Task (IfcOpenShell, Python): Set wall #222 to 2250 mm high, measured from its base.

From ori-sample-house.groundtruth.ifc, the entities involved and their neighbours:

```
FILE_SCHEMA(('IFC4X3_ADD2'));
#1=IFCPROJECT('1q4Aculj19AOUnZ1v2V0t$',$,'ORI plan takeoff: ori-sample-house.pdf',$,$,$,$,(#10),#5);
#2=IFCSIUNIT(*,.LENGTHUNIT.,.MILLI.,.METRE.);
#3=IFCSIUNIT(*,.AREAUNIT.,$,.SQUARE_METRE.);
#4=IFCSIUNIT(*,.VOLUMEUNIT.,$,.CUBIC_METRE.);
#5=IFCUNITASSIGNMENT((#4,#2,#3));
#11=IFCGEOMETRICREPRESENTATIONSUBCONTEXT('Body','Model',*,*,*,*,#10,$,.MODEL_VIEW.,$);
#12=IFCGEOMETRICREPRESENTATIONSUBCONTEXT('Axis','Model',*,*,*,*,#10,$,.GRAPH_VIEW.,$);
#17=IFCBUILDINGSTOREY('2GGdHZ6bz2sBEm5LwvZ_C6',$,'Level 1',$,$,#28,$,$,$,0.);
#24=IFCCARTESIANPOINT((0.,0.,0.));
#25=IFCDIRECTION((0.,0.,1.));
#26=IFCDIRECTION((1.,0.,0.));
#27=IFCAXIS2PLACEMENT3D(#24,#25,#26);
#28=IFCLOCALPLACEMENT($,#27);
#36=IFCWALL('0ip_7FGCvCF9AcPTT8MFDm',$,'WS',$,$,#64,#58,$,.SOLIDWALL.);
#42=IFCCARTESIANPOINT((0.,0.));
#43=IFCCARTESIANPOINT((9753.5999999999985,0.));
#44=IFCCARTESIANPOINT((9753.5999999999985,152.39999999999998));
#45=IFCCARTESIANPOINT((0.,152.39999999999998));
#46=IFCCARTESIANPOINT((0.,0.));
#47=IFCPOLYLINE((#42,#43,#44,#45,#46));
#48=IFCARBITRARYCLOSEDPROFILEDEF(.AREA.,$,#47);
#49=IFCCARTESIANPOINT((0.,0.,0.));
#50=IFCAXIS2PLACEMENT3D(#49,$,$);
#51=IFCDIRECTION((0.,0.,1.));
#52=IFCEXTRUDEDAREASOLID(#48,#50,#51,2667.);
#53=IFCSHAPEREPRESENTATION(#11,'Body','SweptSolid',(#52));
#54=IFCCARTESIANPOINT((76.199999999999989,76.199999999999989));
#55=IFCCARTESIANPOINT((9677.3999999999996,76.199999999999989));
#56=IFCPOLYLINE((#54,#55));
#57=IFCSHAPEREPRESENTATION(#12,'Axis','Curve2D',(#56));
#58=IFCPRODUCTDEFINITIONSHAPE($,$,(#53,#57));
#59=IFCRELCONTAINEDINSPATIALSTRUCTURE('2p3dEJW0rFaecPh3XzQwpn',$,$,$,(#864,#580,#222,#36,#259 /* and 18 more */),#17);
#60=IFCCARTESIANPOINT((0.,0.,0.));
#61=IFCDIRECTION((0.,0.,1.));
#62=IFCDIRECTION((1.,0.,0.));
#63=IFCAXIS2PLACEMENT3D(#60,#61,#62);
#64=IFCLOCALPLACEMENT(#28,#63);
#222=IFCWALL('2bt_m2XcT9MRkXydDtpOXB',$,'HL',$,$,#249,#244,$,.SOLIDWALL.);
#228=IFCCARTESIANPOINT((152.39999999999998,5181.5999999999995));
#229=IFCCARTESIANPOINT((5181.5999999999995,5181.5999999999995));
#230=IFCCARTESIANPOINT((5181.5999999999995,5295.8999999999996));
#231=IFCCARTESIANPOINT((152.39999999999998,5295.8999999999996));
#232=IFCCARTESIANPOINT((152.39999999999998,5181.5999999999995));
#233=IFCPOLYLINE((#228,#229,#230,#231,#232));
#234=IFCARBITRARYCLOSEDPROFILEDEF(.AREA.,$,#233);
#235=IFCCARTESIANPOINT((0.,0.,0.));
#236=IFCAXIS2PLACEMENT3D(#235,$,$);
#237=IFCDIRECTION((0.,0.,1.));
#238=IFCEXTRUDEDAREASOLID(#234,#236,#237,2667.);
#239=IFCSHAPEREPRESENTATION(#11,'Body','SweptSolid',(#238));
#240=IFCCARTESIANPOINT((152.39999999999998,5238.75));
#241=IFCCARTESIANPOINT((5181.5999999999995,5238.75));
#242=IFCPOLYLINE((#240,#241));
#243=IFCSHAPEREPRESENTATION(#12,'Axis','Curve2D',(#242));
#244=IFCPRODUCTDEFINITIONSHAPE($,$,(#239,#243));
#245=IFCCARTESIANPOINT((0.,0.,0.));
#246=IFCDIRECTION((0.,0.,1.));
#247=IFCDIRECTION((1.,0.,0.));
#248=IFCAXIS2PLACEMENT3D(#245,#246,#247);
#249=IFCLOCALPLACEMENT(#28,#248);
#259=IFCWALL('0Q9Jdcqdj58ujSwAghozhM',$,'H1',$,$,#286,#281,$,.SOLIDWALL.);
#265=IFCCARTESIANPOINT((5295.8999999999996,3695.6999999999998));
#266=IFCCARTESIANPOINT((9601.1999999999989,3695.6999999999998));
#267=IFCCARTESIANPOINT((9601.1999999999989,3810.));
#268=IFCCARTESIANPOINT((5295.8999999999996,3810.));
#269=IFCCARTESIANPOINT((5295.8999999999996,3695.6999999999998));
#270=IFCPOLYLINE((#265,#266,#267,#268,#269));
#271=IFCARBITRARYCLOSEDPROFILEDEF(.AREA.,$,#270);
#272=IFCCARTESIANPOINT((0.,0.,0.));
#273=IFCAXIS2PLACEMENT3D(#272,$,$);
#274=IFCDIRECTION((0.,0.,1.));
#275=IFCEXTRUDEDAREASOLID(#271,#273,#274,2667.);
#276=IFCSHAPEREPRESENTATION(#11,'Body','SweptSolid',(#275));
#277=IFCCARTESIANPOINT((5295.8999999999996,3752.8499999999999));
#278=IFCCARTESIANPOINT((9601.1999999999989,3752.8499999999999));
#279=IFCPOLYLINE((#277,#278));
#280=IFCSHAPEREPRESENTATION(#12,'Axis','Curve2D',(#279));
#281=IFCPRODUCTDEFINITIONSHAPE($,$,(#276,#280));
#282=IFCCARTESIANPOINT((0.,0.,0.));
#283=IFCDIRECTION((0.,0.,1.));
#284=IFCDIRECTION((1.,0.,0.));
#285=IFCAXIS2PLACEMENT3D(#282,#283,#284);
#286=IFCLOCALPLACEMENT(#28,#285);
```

```python
import ifcopenshell
import ifcopenshell.geom
import ifcopenshell.util.representation
import ifcopenshell.util.shape

model = ifcopenshell.open("ori-sample-house.groundtruth.ifc")
settings = ifcopenshell.geom.settings()


def volume(element):
    """Net volume in cubic metres, openings subtracted."""
    shape = ifcopenshell.geom.create_shape(settings, element)
    return ifcopenshell.util.shape.get_volume(shape.geometry)


wall = model.by_guid("2bt_m2XcT9MRkXydDtpOXB")
before = volume(wall)

body = ifcopenshell.util.representation.get_representation(wall, "Model", "Body")
solid = body.Items[0]
old_height = solid.Depth
solid.Depth = 2250.0
after = volume(wall)

print(f"height {old_height:g} -> {solid.Depth:g}, volume {before:.3f} -> {after:.3f} m3")

model.write("ori-sample-house.groundtruth-out.ifc")
```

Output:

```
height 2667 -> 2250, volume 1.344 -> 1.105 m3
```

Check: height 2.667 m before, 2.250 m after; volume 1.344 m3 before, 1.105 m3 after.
